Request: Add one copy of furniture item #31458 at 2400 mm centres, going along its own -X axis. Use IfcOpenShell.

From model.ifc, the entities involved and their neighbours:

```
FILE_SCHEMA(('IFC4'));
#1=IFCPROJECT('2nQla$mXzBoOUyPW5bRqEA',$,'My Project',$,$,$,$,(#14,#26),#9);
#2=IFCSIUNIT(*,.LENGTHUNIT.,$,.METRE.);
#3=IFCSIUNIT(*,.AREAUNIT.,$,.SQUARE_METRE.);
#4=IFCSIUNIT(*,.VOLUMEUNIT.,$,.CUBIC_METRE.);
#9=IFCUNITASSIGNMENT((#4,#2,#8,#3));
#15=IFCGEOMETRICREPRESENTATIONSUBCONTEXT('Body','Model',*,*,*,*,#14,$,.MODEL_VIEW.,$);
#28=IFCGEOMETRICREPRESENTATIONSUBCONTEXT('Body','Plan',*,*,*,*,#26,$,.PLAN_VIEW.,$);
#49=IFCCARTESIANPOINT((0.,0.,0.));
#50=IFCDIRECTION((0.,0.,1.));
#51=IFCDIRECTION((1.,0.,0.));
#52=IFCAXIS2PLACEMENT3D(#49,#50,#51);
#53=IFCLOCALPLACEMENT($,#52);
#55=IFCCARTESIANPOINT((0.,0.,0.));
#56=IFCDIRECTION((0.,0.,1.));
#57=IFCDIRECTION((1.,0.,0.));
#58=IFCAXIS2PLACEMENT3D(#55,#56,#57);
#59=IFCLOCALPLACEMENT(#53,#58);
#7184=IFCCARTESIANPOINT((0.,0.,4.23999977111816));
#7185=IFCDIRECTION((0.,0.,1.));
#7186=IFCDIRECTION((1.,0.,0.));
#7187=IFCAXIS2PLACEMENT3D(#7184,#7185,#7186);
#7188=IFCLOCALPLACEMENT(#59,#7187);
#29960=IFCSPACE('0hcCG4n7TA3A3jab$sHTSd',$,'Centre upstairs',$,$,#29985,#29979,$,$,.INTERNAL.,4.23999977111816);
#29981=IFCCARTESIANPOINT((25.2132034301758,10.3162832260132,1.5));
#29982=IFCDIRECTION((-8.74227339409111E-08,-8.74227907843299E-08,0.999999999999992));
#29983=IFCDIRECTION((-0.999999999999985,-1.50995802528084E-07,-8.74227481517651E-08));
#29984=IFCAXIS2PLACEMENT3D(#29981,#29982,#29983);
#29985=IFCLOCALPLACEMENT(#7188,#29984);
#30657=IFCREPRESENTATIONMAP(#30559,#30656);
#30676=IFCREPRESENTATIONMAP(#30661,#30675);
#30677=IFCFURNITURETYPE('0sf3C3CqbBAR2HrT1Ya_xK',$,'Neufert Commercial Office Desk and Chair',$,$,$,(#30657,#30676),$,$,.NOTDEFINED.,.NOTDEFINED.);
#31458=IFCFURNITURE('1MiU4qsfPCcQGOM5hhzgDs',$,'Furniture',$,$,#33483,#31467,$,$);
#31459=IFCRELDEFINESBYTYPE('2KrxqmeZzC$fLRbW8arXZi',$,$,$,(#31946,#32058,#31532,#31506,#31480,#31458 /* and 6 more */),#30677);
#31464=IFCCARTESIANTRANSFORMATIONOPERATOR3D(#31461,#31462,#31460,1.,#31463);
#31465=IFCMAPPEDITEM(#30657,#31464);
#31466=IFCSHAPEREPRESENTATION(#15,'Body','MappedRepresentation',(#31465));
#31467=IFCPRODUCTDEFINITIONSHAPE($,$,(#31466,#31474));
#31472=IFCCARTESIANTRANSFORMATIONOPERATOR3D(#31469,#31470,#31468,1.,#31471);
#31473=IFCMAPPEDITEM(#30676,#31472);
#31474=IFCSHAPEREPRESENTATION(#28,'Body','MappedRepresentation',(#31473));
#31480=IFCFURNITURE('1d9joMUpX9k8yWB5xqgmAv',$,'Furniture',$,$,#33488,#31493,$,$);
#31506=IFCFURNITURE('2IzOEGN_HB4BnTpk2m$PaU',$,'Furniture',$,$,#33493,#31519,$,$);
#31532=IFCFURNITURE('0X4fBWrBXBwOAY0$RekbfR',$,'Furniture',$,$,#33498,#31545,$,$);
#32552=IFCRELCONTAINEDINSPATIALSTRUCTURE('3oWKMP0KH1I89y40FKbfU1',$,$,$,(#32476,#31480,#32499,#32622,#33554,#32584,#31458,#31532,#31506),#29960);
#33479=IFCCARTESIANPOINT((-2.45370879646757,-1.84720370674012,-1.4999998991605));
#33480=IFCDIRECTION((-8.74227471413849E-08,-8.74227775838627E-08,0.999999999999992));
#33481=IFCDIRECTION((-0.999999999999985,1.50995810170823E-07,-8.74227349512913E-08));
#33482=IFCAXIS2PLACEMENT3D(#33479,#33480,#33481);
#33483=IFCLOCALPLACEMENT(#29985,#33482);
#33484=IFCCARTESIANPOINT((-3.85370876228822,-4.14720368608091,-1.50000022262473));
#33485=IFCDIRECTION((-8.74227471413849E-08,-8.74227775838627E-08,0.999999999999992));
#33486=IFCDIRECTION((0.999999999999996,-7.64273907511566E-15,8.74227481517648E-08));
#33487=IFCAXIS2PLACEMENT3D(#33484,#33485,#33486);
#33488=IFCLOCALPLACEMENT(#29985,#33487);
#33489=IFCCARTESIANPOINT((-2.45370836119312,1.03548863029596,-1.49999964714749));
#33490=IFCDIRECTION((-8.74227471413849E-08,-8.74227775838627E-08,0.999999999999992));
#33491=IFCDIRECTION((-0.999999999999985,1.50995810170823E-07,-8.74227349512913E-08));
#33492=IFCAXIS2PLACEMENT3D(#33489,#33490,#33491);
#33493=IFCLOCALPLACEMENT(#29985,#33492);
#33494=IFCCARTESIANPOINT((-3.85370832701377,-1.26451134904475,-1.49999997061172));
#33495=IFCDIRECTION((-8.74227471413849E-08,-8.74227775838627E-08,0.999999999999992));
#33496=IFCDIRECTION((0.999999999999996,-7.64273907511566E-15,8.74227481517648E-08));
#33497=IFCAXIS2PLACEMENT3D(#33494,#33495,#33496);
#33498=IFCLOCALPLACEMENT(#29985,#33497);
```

```python
import ifcopenshell
import ifcopenshell.api.geometry
import ifcopenshell.api.root
import ifcopenshell.util.element
import ifcopenshell.util.placement

model = ifcopenshell.open("model.ifc")

source = model.by_guid("1MiU4qsfPCcQGOM5hhzgDs")
base = ifcopenshell.util.placement.get_local_placement(source.ObjectPlacement)
step = -base[:3, 0] * 2.4

for i in range(1, 2):
    copy = ifcopenshell.api.root.copy_class(model, product=source)
    copy.Representation = ifcopenshell.util.element.copy_deep(
        model, source.Representation, exclude=["IfcGeometricRepresentationContext", "IfcRepresentationMap"]
    )
    matrix = base.copy()
    matrix[:3, 3] += i * step
    print("added at", matrix[:3, 3].round(3) + 0.0)
    ifcopenshell.api.geometry.edit_object_placement(model, product=copy, matrix=matrix, is_si=False)

model.write("model_rev.ifc")
```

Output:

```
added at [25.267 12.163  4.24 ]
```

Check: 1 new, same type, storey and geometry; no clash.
